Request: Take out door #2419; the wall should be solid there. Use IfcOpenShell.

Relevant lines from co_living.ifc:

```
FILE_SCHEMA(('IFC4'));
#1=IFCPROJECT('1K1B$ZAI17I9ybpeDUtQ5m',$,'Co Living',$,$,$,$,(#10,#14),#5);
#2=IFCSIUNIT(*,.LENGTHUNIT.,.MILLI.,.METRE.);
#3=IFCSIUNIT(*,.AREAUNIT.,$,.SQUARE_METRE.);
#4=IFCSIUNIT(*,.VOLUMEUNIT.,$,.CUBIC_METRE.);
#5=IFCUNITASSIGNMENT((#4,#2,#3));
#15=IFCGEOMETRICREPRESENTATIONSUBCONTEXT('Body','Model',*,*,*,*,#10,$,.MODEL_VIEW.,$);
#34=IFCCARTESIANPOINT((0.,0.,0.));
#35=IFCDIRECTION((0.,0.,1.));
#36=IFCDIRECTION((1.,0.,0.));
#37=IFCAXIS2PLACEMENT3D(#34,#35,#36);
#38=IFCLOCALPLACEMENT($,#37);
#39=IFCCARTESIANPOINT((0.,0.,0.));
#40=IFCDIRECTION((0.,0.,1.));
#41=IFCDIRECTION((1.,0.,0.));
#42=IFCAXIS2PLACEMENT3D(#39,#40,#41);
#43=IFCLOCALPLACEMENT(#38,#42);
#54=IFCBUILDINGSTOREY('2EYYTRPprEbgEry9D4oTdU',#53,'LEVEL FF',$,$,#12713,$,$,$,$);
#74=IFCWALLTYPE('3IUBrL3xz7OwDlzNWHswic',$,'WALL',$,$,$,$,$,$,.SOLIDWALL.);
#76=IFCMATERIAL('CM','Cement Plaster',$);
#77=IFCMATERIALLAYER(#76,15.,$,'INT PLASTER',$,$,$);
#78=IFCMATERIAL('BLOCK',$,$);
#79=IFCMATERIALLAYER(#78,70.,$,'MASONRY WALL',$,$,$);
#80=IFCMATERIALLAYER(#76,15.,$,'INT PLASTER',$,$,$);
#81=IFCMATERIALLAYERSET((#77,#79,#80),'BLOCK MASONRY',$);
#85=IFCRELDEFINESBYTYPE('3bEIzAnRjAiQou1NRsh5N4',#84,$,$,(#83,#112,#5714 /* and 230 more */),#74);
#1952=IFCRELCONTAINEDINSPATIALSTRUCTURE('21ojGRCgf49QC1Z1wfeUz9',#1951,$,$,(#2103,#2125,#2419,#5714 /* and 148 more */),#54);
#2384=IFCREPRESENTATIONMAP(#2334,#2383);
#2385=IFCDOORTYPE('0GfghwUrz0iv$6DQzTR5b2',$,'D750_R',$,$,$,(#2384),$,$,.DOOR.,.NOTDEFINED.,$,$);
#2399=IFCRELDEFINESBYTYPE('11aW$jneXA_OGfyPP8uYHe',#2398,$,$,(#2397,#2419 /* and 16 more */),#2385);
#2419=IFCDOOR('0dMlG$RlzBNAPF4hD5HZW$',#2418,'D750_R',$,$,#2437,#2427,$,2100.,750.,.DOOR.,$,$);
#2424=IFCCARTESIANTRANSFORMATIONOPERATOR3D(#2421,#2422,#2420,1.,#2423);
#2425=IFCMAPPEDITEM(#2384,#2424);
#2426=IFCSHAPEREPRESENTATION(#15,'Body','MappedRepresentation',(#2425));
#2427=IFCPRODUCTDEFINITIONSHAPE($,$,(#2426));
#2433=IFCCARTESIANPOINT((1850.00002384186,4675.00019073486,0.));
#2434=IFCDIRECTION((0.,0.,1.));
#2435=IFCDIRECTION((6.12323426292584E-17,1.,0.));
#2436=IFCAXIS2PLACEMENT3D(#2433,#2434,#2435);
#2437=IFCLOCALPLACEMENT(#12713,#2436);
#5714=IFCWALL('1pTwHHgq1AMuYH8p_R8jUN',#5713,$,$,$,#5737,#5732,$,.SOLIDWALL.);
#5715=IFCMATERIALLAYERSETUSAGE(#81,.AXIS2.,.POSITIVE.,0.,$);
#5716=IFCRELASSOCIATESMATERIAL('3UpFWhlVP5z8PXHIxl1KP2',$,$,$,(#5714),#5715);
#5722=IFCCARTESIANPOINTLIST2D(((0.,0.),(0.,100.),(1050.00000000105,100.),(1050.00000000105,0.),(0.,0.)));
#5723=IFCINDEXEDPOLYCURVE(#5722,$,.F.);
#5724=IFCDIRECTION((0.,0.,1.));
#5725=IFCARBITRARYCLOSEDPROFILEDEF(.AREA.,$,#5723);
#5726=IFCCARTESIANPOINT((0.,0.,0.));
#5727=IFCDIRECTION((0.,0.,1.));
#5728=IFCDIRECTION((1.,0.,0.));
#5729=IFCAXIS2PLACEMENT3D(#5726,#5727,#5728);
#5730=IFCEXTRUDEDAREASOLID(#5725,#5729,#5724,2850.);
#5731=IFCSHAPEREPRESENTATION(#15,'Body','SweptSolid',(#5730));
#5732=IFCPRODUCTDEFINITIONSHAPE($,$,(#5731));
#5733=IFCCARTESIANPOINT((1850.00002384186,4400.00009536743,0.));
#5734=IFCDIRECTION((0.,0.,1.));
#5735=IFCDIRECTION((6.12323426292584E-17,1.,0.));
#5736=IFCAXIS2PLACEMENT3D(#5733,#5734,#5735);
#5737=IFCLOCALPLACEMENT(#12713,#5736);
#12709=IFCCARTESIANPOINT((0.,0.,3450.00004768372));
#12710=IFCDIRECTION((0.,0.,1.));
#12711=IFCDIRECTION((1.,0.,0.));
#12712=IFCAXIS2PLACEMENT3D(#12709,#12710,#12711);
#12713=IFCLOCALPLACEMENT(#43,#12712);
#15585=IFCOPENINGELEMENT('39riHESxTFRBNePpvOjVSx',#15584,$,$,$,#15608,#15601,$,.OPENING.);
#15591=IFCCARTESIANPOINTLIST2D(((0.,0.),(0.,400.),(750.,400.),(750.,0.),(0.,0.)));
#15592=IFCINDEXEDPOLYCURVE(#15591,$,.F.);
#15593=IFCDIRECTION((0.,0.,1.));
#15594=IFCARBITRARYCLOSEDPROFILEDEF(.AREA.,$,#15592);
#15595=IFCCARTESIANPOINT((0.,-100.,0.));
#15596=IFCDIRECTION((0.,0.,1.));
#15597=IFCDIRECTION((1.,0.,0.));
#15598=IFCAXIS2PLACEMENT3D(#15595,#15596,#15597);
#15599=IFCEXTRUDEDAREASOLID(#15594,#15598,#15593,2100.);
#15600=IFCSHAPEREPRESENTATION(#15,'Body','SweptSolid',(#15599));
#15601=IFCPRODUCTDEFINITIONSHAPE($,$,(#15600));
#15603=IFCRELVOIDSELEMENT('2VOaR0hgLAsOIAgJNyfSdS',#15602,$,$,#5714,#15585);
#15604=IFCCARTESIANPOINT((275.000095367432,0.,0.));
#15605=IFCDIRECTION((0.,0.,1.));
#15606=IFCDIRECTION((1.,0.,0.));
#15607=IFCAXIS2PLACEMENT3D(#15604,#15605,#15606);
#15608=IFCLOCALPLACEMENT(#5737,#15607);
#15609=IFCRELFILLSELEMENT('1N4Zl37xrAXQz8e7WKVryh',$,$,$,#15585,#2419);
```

```python
import ifcopenshell
import ifcopenshell.api.feature
import ifcopenshell.api.root
import ifcopenshell.geom
import ifcopenshell.util.shape

model = ifcopenshell.open("co_living.ifc")
settings = ifcopenshell.geom.settings()


def volume(element):
    """Net volume in cubic metres, openings subtracted."""
    shape = ifcopenshell.geom.create_shape(settings, element)
    return ifcopenshell.util.shape.get_volume(shape.geometry)


door = model.by_guid("0dMlG$RlzBNAPF4hD5HZW$")
opening = door.FillsVoids[0].RelatingOpeningElement
wall = opening.VoidsElements[0].RelatingBuildingElement
before = volume(wall)

ifcopenshell.api.root.remove_product(model, product=door)
ifcopenshell.api.feature.remove_feature(model, feature=opening)

after = volume(wall)

print(f"wall volume {before:.3f} -> {after:.3f} m3")

model.write("co_living_edited.ifc")
```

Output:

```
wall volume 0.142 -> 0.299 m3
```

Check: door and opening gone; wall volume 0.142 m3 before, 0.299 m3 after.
